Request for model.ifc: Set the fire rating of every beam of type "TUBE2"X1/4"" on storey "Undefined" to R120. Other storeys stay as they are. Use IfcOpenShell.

First a look at what the model holds.

```python
import ifcopenshell
import ifcopenshell.util.element

model = ifcopenshell.open("model.ifc")
print(model.schema)
storey = next(s for s in model.by_type("IfcBuildingStorey") if s.Name == "Undefined")
beams = [e for e in ifcopenshell.util.element.get_decomposition(storey) if e.is_a("IfcBeam")]
seen = {}
for e in beams:
    element_type = ifcopenshell.util.element.get_type(e)
    key = (element_type.Name if element_type != e and element_type else None, ifcopenshell.util.element.get_pset(e, "Pset_BeamCommon", "FireRating"))
    seen[key] = seen.get(key, 0) + 1
for (name, value), count in sorted(seen.items(), key=str):
    print(count, "x", name, "|", value)
```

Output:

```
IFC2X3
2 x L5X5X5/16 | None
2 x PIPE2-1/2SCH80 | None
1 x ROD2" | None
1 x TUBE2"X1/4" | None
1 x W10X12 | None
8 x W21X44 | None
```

```python
import ifcopenshell
import ifcopenshell.api.pset
import ifcopenshell.util.element

model = ifcopenshell.open("model.ifc")

storey = next(s for s in model.by_type("IfcBuildingStorey") if s.Name == "Undefined")
beams = [e for e in ifcopenshell.util.element.get_decomposition(storey) if e.is_a("IfcBeam")]

count = 0
for e in beams:
    element_type = ifcopenshell.util.element.get_type(e)
    if element_type in (None, e) or element_type.Name != 'TUBE2"X1/4"':
        continue
    # add_pset returns the element's existing set when there is one.
    pset = ifcopenshell.api.pset.add_pset(model, product=e, name="Pset_BeamCommon")
    ifcopenshell.api.pset.edit_pset(model, pset=pset, properties={"FireRating": "R120"})
    count += 1

print(count, "beams updated")

model.write("model_v2.ifc")
```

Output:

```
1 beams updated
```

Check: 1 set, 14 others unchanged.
